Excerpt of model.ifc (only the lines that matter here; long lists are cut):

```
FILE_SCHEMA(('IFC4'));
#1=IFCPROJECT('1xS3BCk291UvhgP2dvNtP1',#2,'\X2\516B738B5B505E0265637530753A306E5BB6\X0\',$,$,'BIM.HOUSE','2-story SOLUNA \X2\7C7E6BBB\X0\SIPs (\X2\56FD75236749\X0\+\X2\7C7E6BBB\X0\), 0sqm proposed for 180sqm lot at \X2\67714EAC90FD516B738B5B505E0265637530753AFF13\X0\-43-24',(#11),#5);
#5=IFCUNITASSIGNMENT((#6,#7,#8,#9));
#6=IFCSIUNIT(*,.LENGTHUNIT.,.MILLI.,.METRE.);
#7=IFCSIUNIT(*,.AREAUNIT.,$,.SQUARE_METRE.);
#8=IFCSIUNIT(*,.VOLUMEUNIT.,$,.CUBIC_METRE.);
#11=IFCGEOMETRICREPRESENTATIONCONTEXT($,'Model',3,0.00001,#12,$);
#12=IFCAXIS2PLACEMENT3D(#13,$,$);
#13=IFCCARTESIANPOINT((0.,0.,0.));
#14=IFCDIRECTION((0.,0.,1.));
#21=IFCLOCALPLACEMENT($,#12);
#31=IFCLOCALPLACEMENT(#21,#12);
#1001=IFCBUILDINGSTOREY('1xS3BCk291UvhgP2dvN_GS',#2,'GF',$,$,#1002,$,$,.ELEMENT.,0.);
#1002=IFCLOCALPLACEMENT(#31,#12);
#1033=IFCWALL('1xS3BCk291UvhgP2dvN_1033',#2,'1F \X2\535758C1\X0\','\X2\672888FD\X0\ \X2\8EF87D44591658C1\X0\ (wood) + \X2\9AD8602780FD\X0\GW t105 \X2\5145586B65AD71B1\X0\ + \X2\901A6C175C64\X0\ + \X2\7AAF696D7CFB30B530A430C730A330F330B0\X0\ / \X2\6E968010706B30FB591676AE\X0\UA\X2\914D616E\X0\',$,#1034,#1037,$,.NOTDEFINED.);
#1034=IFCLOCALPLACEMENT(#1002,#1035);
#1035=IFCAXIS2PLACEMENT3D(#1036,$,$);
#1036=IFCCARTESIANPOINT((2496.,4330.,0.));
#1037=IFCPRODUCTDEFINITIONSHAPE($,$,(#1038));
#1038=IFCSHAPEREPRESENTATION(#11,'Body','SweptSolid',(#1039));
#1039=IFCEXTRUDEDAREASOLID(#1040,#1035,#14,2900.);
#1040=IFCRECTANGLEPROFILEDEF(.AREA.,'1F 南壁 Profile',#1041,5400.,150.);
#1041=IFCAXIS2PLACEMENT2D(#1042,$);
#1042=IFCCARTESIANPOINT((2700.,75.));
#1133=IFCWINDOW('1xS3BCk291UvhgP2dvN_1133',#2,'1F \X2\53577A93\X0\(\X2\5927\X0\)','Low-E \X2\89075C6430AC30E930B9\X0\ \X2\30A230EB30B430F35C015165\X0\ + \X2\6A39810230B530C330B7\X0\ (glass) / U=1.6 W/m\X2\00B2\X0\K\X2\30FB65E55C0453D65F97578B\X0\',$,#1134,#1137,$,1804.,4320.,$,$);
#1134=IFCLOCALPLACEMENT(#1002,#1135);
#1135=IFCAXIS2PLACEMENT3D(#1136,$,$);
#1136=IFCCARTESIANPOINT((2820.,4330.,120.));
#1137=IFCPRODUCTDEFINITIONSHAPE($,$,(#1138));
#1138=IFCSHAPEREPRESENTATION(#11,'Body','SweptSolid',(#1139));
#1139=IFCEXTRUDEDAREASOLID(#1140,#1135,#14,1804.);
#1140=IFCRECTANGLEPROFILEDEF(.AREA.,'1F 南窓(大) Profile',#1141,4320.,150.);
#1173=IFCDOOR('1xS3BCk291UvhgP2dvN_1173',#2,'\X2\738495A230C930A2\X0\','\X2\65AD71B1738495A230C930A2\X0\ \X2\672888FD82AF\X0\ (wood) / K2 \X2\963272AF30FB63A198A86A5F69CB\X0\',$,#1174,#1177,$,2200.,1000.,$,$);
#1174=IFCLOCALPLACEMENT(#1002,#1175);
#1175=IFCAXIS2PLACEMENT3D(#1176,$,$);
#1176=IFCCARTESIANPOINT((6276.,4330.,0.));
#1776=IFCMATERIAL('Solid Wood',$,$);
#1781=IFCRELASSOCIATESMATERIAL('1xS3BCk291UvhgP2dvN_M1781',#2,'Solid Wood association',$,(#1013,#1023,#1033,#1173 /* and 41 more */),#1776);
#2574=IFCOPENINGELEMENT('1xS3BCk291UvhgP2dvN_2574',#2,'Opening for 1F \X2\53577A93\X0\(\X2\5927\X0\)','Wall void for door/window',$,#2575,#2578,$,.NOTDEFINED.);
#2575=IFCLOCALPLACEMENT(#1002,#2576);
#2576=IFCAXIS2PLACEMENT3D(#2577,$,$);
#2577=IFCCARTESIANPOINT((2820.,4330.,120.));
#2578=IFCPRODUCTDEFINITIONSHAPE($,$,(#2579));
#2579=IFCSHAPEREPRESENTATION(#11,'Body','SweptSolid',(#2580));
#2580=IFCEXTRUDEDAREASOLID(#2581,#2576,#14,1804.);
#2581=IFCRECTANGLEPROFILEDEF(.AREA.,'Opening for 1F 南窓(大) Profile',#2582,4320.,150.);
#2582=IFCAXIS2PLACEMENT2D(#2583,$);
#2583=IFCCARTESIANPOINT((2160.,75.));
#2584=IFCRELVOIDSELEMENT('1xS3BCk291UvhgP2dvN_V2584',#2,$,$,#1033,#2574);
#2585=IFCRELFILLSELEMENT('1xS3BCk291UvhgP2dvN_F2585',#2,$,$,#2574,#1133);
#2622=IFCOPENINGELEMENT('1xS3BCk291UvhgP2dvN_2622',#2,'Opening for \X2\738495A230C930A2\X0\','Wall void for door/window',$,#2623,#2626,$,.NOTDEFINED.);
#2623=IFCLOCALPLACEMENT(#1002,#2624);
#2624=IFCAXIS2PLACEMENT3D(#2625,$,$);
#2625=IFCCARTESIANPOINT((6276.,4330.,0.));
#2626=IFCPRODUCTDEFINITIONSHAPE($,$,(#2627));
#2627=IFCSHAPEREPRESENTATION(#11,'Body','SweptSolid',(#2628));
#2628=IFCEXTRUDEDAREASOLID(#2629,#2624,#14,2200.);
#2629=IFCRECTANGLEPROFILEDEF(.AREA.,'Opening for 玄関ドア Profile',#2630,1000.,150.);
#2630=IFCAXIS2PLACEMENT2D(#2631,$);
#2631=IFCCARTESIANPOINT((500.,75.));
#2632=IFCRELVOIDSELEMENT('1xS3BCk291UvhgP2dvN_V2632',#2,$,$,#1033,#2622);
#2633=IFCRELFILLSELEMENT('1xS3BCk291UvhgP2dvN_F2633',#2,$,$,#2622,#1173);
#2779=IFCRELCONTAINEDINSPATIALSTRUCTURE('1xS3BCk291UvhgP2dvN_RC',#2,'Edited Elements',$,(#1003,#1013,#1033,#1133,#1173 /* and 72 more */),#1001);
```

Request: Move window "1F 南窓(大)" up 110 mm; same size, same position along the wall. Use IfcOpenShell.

```python
import numpy as np
import ifcopenshell
import ifcopenshell.api.geometry
import ifcopenshell.util.placement
import ifcopenshell.util.unit

model = ifcopenshell.open("model.ifc")
unit_scale = ifcopenshell.util.unit.calculate_unit_scale(model)

window = model.by_id(1133)
opening = window.FillsVoids[0].RelatingOpeningElement
dz = 0.11 / unit_scale

shift = np.array([0.0, 0.0, dz])
# The window is not placed relative to its opening, so move both.
for product in (opening, window):
    matrix = ifcopenshell.util.placement.get_local_placement(product.ObjectPlacement)
    matrix[:3, 3] += shift
    ifcopenshell.api.geometry.edit_object_placement(model, product=product, matrix=matrix, is_si=False)

print(f"moved by {dz * unit_scale:+.3f} m")

model.write("model_rev.ifc")
```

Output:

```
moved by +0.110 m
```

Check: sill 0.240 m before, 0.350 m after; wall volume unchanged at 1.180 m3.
